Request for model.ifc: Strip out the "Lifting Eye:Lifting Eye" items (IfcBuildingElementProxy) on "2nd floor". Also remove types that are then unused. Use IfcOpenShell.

First a look at what the model holds.

```python
import ifcopenshell
import ifcopenshell.util.element

model = ifcopenshell.open("model.ifc")
print(model.schema)
storey = next(s for s in model.by_type("IfcBuildingStorey") if s.Name == "2nd floor")
proxies = [e for e in ifcopenshell.util.element.get_decomposition(storey) if e.is_a("IfcBuildingElementProxy")]
seen = {}
for e in proxies:
    element_type = ifcopenshell.util.element.get_type(e)
    name = element_type.Name if element_type not in (None, e) else None
    seen[name] = seen.get(name, 0) + 1
for name, count in sorted(seen.items(), key=str):
    print(count, "x", name)
```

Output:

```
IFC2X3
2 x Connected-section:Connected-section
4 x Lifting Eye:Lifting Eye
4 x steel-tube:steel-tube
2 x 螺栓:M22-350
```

```python
import ifcopenshell
import ifcopenshell.api.root
import ifcopenshell.util.element

model = ifcopenshell.open("model.ifc")

storey = next(s for s in model.by_type("IfcBuildingStorey") if s.Name == "2nd floor")
proxies = [e for e in ifcopenshell.util.element.get_decomposition(storey) if e.is_a("IfcBuildingElementProxy")]
targets = [e for e in proxies if (t := ifcopenshell.util.element.get_type(e)) not in (None, e) and t.Name == "Lifting Eye:Lifting Eye"]
types = {ifcopenshell.util.element.get_type(e) for e in targets} - {None, *targets}

for e in targets:
    ifcopenshell.api.root.remove_product(model, product=e)
print(len(targets), "removed")

unused = [t for t in types if not ifcopenshell.util.element.get_types(t)]
for t in unused:
    ifcopenshell.api.root.remove_product(model, product=t)
print(len(unused), "unused types removed")

model.write("model_v2.ifc")
```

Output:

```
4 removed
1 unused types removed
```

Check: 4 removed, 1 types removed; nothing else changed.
